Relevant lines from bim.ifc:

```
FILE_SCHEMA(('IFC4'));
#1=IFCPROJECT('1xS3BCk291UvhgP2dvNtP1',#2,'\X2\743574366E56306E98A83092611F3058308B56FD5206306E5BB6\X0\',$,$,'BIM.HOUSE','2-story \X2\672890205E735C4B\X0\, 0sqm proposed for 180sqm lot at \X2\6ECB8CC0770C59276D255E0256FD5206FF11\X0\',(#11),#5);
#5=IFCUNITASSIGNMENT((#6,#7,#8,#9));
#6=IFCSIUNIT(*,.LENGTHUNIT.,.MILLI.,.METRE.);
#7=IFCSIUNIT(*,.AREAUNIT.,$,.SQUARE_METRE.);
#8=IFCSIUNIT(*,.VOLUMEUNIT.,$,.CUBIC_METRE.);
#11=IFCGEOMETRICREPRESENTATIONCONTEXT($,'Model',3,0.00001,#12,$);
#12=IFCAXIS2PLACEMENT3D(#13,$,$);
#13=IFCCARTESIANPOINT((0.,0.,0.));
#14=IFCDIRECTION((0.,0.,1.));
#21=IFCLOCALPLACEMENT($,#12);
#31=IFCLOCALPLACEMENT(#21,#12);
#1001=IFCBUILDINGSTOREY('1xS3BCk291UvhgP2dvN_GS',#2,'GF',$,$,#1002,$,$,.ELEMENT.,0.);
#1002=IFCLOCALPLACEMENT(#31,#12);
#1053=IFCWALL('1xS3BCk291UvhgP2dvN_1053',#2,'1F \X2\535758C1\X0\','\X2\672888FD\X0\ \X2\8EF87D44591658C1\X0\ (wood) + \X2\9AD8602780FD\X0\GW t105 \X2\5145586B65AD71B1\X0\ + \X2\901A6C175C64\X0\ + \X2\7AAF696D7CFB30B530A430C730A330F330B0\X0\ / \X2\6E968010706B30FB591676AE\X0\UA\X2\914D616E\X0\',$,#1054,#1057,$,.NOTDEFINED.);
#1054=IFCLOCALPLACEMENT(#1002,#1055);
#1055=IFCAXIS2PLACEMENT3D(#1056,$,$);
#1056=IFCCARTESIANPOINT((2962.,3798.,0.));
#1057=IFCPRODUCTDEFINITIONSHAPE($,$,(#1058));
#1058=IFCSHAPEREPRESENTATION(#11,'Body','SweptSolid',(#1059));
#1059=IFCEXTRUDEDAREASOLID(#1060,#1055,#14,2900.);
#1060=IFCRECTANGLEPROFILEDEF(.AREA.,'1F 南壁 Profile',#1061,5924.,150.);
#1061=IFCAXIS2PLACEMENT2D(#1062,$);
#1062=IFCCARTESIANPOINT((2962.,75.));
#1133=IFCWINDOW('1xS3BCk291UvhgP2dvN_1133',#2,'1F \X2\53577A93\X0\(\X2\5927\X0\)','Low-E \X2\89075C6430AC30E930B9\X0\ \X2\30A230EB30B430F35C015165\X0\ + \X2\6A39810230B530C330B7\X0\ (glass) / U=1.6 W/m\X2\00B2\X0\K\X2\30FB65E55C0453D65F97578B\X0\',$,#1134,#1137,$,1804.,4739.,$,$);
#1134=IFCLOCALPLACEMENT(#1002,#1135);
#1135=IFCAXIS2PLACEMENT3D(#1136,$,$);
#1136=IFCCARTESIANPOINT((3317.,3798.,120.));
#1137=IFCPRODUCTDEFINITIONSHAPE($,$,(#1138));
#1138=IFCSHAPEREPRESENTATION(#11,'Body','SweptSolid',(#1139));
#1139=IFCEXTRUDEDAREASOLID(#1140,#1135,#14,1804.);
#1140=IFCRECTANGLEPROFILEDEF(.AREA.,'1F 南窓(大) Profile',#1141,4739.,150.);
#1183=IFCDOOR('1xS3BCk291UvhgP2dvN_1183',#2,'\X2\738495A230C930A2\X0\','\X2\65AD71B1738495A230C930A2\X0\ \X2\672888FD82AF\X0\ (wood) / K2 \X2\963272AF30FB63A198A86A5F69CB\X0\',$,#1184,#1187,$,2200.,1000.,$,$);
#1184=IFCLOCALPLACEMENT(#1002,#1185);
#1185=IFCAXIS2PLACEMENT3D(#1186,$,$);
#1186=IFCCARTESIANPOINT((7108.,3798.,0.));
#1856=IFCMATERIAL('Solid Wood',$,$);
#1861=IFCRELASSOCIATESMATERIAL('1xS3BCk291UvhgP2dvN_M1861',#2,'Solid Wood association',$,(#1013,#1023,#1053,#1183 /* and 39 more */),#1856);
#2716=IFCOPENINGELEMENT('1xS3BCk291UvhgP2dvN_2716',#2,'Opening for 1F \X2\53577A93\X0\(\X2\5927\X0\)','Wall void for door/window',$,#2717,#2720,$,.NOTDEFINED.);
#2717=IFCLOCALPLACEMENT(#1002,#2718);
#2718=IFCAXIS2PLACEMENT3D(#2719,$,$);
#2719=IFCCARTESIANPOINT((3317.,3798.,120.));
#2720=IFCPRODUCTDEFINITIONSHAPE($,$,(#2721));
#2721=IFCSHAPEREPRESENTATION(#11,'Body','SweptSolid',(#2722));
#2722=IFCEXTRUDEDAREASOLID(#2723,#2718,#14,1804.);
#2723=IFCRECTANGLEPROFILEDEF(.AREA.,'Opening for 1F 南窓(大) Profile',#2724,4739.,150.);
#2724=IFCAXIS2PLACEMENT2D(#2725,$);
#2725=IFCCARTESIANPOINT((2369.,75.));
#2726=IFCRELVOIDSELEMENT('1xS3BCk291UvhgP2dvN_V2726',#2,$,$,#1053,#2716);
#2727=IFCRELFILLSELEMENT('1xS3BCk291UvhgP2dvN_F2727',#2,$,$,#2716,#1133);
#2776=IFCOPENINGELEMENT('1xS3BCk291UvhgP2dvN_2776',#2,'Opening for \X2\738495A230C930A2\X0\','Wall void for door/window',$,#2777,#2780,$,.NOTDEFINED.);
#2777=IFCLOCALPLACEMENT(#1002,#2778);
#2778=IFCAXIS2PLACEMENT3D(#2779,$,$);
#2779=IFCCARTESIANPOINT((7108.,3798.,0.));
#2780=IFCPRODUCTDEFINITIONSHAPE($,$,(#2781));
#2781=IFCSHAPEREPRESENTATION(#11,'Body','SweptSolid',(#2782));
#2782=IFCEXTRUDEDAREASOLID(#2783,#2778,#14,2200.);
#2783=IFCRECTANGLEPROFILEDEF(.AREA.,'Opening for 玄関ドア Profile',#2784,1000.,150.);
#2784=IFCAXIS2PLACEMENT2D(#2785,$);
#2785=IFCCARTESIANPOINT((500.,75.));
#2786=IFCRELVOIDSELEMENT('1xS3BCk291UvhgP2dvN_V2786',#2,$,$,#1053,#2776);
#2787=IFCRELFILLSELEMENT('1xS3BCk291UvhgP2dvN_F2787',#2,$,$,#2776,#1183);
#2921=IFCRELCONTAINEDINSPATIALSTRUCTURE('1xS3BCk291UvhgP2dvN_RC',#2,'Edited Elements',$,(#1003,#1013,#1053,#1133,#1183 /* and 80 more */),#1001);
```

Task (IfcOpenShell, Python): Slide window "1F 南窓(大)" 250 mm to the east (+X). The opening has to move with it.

```python
import ifcopenshell
import ifcopenshell.api.geometry
import ifcopenshell.util.placement
import ifcopenshell.util.unit

model = ifcopenshell.open("bim.ifc")
unit_scale = ifcopenshell.util.unit.calculate_unit_scale(model)

window = model.by_id(1133)
opening = window.FillsVoids[0].RelatingOpeningElement
wall = opening.VoidsElements[0].RelatingBuildingElement

wall_matrix = ifcopenshell.util.placement.get_local_placement(wall.ObjectPlacement)
shift = wall_matrix[:3, 0] * 0.25 / unit_scale
before = ifcopenshell.util.placement.get_local_placement(window.ObjectPlacement)[:3, 3].copy()

# The window is not placed relative to its opening, so move both.
for product in (opening, window):
    matrix = ifcopenshell.util.placement.get_local_placement(product.ObjectPlacement)
    matrix[:3, 3] += shift
    ifcopenshell.api.geometry.edit_object_placement(model, product=product, matrix=matrix, is_si=False)

after = ifcopenshell.util.placement.get_local_placement(window.ObjectPlacement)[:3, 3]
print("window moved by", (after - before).round(3) + 0.0)

model.write("bim_edited.ifc")
```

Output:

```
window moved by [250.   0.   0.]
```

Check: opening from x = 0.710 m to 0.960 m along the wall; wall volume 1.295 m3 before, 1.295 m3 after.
